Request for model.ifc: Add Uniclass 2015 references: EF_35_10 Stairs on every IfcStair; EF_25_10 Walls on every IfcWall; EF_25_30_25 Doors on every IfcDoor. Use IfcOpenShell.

First a look at what the model holds.

```python
import ifcopenshell

model = ifcopenshell.open("model.ifc")
print(model.schema)
print("classifications:", [c.Name for c in model.by_type("IfcClassification")])
for ifc_class in ("IfcDoor", "IfcRoof", "IfcStair", "IfcWall", "IfcWindow"):
    print(ifc_class, len(model.by_type(ifc_class)))
```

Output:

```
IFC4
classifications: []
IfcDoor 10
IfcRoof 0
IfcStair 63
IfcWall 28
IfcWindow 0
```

```python
import ifcopenshell
import ifcopenshell.api.classification

model = ifcopenshell.open("model.ifc")

system = ifcopenshell.api.classification.add_classification(model, classification="Uniclass 2015")

codes = {
    "IfcStair": ("EF_35_10", "Stairs"),
    "IfcWall": ("EF_25_10", "Walls"),
    "IfcDoor": ("EF_25_30_25", "Doors"),
}
for ifc_class, (code, name) in codes.items():
    products = model.by_type(ifc_class)
    ifcopenshell.api.classification.add_reference(
        model, products=products, classification=system, identification=code, name=name
    )
    print(code, len(products))

model.write("model_v2.ifc")
```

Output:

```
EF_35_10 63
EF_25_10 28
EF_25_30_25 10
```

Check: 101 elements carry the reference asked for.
